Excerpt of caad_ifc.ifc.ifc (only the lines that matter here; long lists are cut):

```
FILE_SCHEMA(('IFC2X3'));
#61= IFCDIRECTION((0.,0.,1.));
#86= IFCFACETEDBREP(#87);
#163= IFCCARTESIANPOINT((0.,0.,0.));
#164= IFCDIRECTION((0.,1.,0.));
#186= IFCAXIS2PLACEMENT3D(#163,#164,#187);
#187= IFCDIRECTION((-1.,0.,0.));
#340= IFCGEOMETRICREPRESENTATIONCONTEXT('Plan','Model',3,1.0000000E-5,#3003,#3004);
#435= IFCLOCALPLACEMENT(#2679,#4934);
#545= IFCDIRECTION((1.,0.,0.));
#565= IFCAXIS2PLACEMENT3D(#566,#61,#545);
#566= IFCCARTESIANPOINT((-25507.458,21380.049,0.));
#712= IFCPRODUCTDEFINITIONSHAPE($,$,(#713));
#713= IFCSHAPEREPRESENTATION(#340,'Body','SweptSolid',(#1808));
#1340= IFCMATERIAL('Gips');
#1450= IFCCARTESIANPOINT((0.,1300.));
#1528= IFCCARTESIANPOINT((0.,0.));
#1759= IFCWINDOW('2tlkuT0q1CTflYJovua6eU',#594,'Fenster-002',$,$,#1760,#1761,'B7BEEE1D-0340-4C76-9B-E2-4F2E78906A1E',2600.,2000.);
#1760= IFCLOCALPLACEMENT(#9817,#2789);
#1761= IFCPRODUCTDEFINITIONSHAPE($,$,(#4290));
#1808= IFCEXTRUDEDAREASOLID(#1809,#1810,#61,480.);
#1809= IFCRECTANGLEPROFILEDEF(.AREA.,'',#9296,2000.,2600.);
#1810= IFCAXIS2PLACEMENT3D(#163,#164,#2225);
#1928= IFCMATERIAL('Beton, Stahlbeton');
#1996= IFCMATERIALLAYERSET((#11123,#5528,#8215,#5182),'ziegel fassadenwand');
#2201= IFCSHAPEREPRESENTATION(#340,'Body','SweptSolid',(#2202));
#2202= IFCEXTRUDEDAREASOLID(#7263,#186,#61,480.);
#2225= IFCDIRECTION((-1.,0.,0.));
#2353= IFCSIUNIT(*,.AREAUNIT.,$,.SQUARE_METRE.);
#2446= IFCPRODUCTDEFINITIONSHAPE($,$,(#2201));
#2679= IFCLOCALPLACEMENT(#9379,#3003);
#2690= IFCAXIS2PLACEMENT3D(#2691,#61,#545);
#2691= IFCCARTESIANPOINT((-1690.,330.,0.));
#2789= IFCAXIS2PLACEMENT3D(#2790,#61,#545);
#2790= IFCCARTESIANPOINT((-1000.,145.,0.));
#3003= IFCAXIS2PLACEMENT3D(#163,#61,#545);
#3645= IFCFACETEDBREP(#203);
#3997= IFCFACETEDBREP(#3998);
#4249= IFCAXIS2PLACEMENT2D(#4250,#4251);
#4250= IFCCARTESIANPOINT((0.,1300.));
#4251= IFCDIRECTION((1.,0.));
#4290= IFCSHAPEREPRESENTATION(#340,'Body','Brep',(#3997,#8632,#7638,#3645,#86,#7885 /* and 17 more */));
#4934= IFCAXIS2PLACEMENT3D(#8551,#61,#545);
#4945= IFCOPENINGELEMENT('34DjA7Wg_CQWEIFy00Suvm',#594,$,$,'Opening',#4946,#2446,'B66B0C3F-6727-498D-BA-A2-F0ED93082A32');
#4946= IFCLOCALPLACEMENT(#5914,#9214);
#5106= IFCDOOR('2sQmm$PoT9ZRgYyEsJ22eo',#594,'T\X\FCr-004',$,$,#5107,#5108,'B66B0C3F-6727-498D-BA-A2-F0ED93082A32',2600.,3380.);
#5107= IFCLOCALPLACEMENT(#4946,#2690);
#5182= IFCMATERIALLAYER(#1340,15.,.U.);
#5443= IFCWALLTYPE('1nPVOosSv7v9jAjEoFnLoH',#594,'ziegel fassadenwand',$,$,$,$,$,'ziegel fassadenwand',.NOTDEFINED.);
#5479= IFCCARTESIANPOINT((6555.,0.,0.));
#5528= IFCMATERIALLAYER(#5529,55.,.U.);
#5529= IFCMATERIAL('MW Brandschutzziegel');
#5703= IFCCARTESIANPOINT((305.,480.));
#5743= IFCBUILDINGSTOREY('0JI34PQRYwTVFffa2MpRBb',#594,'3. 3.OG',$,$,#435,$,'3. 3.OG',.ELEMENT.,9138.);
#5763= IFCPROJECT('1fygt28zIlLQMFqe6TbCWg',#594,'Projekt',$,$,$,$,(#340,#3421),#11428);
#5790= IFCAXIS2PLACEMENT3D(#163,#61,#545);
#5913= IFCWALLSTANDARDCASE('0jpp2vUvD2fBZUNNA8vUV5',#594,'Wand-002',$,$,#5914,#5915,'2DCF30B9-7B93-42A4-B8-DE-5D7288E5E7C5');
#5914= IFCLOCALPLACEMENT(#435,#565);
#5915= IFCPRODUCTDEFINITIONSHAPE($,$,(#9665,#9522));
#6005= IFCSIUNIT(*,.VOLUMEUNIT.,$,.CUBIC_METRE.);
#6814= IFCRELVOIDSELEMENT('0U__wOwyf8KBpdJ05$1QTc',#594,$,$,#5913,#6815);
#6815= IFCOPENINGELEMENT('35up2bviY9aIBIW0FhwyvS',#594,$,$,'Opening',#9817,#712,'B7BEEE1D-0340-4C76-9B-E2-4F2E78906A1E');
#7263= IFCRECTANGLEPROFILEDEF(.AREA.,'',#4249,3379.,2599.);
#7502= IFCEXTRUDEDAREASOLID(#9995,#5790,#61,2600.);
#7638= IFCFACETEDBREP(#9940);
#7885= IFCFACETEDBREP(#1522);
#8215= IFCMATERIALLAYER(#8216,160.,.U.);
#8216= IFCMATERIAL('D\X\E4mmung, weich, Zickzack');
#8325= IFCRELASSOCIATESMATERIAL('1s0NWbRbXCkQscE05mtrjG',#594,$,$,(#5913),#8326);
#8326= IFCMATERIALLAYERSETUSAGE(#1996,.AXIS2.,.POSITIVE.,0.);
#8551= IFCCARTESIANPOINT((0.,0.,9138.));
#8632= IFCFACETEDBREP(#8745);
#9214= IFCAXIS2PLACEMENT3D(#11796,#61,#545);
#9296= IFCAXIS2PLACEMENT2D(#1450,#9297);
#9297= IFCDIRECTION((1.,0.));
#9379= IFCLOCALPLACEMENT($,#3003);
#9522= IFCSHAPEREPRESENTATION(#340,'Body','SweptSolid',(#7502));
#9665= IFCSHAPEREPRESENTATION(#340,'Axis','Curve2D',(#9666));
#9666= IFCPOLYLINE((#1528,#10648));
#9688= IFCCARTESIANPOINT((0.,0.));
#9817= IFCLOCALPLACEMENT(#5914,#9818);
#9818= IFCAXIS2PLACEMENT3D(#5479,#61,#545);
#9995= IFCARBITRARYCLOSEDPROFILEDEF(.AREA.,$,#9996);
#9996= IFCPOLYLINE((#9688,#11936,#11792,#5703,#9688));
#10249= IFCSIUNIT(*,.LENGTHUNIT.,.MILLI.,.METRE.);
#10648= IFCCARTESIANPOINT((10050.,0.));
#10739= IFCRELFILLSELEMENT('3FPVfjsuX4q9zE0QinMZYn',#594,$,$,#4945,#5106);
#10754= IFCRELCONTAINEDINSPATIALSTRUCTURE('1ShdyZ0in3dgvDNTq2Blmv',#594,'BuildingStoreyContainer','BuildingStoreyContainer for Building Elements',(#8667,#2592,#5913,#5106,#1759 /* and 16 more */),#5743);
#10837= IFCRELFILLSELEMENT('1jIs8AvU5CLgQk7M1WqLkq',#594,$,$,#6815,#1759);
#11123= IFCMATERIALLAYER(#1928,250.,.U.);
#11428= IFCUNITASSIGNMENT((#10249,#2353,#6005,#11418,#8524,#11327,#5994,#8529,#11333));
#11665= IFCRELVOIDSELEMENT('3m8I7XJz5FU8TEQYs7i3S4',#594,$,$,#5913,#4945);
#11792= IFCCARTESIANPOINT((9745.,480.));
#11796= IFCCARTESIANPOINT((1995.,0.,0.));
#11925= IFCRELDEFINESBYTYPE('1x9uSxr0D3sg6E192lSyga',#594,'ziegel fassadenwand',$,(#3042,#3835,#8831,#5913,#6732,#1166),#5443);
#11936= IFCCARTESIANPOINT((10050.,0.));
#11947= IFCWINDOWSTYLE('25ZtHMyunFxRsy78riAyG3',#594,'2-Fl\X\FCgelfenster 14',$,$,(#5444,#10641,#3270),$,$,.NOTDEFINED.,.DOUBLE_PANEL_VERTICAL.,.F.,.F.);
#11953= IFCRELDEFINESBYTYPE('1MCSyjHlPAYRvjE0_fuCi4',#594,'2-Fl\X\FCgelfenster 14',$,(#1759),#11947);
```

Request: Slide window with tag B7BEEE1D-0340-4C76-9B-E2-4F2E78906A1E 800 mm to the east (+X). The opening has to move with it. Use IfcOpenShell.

```python
import ifcopenshell
import ifcopenshell.api.geometry
import ifcopenshell.util.placement

model = ifcopenshell.open("caad_ifc.ifc.ifc")

window = model.by_id(1759)
opening = window.FillsVoids[0].RelatingOpeningElement
wall = opening.VoidsElements[0].RelatingBuildingElement

wall_matrix = ifcopenshell.util.placement.get_local_placement(wall.ObjectPlacement)
shift = wall_matrix[:3, 0] * 800.0
before = ifcopenshell.util.placement.get_local_placement(window.ObjectPlacement)[:3, 3].copy()

# The window is placed relative to its opening, so it follows when the opening moves.
matrix = ifcopenshell.util.placement.get_local_placement(opening.ObjectPlacement)
matrix[:3, 3] += shift
ifcopenshell.api.geometry.edit_object_placement(
    model, product=opening, matrix=matrix, is_si=False, should_transform_children=True
)

after = ifcopenshell.util.placement.get_local_placement(window.ObjectPlacement)[:3, 3]
print("window moved by", (after - before).round(3) + 0.0)

model.write("caad_ifc.ifc_edited.ifc")
```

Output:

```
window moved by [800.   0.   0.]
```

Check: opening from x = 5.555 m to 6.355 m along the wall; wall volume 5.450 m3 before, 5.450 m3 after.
